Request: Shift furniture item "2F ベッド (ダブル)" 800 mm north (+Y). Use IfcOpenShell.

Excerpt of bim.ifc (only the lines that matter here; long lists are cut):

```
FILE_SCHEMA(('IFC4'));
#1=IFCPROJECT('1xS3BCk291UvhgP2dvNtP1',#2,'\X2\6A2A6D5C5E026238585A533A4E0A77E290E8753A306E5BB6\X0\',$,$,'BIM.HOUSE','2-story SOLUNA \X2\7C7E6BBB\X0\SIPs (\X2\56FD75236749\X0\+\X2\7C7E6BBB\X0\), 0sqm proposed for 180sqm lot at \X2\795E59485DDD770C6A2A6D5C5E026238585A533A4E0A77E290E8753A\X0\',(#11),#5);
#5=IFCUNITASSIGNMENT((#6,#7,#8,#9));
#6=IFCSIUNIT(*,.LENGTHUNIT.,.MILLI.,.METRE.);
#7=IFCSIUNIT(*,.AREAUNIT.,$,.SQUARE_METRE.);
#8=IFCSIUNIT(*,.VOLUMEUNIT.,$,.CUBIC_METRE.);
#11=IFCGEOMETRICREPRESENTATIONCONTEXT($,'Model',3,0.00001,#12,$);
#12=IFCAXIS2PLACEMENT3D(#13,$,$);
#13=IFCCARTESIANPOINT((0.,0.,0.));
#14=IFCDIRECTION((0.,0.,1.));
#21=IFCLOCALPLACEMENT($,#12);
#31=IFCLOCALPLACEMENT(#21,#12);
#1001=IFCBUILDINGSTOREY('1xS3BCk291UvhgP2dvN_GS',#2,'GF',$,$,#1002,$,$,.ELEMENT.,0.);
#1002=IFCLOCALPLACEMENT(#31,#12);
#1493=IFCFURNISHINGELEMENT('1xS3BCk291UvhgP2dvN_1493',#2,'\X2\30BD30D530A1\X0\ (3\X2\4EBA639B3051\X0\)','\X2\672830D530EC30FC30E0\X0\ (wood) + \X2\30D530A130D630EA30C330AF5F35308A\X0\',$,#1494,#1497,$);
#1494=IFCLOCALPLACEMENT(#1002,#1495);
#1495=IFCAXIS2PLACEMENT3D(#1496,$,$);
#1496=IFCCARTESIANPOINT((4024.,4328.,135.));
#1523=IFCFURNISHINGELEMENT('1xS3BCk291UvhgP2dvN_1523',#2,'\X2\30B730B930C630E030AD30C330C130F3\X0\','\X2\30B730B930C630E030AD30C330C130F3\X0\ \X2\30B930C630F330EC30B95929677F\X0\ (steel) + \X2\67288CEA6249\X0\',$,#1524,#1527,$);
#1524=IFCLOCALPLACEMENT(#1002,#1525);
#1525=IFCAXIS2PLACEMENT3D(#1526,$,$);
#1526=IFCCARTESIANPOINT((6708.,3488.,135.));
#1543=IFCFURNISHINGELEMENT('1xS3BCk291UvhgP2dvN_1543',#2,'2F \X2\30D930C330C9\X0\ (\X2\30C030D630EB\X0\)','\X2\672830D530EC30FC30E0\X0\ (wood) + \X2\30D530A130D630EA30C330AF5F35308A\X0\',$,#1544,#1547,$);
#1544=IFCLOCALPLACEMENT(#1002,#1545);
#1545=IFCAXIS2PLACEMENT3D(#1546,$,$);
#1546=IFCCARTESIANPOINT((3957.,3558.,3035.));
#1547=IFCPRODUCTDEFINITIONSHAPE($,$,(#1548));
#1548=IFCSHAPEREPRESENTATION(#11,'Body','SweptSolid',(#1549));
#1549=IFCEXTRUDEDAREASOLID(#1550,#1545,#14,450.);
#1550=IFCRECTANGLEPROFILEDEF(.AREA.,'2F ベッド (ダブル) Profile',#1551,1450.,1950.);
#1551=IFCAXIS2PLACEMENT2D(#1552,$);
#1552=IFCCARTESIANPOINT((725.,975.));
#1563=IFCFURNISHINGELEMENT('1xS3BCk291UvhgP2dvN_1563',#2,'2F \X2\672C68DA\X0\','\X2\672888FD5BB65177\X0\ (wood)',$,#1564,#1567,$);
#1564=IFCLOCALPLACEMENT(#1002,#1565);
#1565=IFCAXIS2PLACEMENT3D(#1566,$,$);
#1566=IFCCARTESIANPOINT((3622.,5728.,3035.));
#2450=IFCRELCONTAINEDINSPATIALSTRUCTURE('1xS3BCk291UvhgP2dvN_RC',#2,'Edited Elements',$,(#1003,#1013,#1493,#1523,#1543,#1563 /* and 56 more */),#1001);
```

```python
import ifcopenshell
import ifcopenshell.api.geometry
import ifcopenshell.util.placement
import ifcopenshell.util.unit

model = ifcopenshell.open("bim.ifc")
unit_scale = ifcopenshell.util.unit.calculate_unit_scale(model)

item = model.by_guid("1xS3BCk291UvhgP2dvN_1543")
matrix = ifcopenshell.util.placement.get_local_placement(item.ObjectPlacement)
matrix[1, 3] += 0.8 / unit_scale
ifcopenshell.api.geometry.edit_object_placement(model, product=item, matrix=matrix, is_si=False)

print(ifcopenshell.util.placement.get_local_placement(item.ObjectPlacement).round(3) + 0.0)

model.write("bim_v2.ifc")
```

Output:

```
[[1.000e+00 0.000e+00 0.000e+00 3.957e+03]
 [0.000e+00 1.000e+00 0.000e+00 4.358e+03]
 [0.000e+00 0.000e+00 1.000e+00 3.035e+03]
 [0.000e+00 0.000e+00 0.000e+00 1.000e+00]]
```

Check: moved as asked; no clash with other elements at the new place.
